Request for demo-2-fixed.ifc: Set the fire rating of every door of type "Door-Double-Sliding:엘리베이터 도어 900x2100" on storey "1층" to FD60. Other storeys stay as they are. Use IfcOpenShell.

First a look at what the model holds.

```python
import ifcopenshell
import ifcopenshell.util.element

model = ifcopenshell.open("demo-2-fixed.ifc")
print(model.schema)
storey = next(s for s in model.by_type("IfcBuildingStorey") if s.Name == "1층")
doors = [e for e in ifcopenshell.util.element.get_decomposition(storey) if e.is_a("IfcDoor")]
seen = {}
for e in doors:
    element_type = ifcopenshell.util.element.get_type(e)
    key = (element_type.Name if element_type != e and element_type else None, ifcopenshell.util.element.get_pset(e, "Pset_DoorCommon", "FireRating"))
    seen[key] = seen.get(key, 0) + 1
for (name, value), count in sorted(seen.items(), key=str):
    print(count, "x", name, "|", value)
```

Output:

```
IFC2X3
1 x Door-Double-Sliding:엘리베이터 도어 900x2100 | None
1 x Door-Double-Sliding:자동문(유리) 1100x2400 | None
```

```python
import ifcopenshell
import ifcopenshell.api.pset
import ifcopenshell.util.element

model = ifcopenshell.open("demo-2-fixed.ifc")

storey = next(s for s in model.by_type("IfcBuildingStorey") if s.Name == "1층")
doors = [e for e in ifcopenshell.util.element.get_decomposition(storey) if e.is_a("IfcDoor")]

count = 0
for e in doors:
    element_type = ifcopenshell.util.element.get_type(e)
    if element_type in (None, e) or element_type.Name != "Door-Double-Sliding:엘리베이터 도어 900x2100":
        continue
    # add_pset returns the element's existing set when there is one.
    pset = ifcopenshell.api.pset.add_pset(model, product=e, name="Pset_DoorCommon")
    ifcopenshell.api.pset.edit_pset(model, pset=pset, properties={"FireRating": "FD60"})
    count += 1

print(count, "doors updated")

model.write("demo-2-fixed-out.ifc")
```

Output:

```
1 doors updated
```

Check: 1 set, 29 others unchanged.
